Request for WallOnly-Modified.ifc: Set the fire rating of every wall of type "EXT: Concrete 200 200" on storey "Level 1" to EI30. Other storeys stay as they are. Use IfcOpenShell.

First a look at what the model holds.

```python
import ifcopenshell
import ifcopenshell.util.element

model = ifcopenshell.open("WallOnly-Modified.ifc")
print(model.schema)
storey = next(s for s in model.by_type("IfcBuildingStorey") if s.Name == "Level 1")
walls = [e for e in ifcopenshell.util.element.get_decomposition(storey) if e.is_a("IfcWall")]
seen = {}
for e in walls:
    element_type = ifcopenshell.util.element.get_type(e)
    key = (element_type.Name if element_type != e and element_type else None, ifcopenshell.util.element.get_pset(e, "Pset_WallCommon", "FireRating"))
    seen[key] = seen.get(key, 0) + 1
for (name, value), count in sorted(seen.items(), key=str):
    print(count, "x", name, "|", value)
```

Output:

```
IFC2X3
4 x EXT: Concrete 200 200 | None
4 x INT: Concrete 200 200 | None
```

```python
import ifcopenshell
import ifcopenshell.api.pset
import ifcopenshell.util.element

model = ifcopenshell.open("WallOnly-Modified.ifc")

storey = next(s for s in model.by_type("IfcBuildingStorey") if s.Name == "Level 1")
walls = [e for e in ifcopenshell.util.element.get_decomposition(storey) if e.is_a("IfcWall")]

count = 0
for e in walls:
    element_type = ifcopenshell.util.element.get_type(e)
    if element_type in (None, e) or element_type.Name != "EXT: Concrete 200 200":
        continue
    # add_pset returns the element's existing set when there is one.
    pset = ifcopenshell.api.pset.add_pset(model, product=e, name="Pset_WallCommon")
    ifcopenshell.api.pset.edit_pset(model, pset=pset, properties={"FireRating": "EI30"})
    count += 1

print(count, "walls updated")

model.write("WallOnly-Modified_v2.ifc")
```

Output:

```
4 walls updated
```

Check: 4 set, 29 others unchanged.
